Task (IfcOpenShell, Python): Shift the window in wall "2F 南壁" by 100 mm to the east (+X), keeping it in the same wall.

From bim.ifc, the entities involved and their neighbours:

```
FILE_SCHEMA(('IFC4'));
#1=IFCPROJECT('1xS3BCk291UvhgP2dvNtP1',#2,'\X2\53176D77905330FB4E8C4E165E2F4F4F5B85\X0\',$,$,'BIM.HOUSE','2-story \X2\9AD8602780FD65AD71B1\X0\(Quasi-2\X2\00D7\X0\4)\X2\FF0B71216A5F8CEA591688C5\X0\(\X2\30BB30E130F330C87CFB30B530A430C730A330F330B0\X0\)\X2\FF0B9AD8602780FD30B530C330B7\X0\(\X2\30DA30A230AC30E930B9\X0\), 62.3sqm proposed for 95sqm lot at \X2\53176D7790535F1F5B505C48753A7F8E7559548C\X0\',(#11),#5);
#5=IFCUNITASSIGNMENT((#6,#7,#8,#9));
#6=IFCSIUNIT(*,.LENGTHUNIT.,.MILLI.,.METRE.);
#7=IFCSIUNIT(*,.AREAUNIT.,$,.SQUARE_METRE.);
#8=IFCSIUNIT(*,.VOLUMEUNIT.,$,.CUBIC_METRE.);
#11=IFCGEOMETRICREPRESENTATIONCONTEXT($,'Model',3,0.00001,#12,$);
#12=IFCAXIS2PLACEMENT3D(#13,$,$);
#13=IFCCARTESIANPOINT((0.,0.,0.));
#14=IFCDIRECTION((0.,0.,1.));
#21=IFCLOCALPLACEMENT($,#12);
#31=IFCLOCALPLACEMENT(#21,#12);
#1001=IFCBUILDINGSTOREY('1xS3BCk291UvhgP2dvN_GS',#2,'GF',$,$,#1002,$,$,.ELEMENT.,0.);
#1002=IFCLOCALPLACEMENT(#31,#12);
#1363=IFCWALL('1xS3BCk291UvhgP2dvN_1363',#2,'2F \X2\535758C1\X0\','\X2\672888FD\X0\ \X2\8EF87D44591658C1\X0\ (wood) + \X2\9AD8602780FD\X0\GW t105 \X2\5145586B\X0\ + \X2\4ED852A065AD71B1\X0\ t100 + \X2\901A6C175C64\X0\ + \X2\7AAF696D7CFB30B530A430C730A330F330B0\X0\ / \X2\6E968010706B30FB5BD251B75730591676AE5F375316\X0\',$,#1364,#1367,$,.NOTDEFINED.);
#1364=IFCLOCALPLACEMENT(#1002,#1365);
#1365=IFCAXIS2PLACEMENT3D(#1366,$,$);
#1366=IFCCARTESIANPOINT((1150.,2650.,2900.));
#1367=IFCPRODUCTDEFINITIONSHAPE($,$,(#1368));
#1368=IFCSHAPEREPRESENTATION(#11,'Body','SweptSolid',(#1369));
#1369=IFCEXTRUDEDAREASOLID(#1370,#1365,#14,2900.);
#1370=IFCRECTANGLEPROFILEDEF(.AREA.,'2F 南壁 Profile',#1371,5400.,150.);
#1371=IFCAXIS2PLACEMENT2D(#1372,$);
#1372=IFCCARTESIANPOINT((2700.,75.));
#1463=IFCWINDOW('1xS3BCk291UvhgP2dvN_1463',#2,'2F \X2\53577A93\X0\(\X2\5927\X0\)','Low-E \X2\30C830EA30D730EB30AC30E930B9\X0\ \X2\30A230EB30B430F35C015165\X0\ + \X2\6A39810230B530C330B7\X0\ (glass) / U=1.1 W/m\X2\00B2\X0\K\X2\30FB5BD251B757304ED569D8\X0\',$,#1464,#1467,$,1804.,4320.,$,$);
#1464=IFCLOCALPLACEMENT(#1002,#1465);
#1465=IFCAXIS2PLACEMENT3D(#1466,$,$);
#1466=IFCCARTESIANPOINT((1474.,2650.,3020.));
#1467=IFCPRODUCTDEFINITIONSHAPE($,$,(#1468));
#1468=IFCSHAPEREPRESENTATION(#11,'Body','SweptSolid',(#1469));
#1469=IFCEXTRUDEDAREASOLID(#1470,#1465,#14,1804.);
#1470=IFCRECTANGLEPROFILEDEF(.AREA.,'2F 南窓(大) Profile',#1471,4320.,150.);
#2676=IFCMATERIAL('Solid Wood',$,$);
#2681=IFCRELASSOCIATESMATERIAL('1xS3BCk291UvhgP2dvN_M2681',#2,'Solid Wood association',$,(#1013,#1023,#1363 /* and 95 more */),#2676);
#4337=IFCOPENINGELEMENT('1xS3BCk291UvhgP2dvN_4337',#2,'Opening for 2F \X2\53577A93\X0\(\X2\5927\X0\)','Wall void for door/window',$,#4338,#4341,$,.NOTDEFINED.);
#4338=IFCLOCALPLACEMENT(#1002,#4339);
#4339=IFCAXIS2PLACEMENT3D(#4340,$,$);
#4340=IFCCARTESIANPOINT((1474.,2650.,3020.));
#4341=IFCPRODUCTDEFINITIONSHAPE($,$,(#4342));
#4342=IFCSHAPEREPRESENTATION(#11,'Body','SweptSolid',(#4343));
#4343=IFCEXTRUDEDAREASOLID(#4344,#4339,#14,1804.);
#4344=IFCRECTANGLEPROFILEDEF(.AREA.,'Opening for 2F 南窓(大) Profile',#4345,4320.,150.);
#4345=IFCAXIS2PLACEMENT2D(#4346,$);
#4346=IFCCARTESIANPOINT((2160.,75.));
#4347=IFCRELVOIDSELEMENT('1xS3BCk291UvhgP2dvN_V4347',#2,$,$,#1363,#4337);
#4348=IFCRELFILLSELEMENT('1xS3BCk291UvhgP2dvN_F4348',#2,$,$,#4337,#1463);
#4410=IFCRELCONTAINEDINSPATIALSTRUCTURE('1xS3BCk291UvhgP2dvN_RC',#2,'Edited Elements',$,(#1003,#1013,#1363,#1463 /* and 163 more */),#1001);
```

```python
import ifcopenshell
import ifcopenshell.api.geometry
import ifcopenshell.util.placement

model = ifcopenshell.open("bim.ifc")

window = model.by_guid("1xS3BCk291UvhgP2dvN_1463")
opening = window.FillsVoids[0].RelatingOpeningElement
wall = opening.VoidsElements[0].RelatingBuildingElement

wall_matrix = ifcopenshell.util.placement.get_local_placement(wall.ObjectPlacement)
shift = wall_matrix[:3, 0] * 100.0
before = ifcopenshell.util.placement.get_local_placement(window.ObjectPlacement)[:3, 3].copy()

# The window is not placed relative to its opening, so move both.
for product in (opening, window):
    matrix = ifcopenshell.util.placement.get_local_placement(product.ObjectPlacement)
    matrix[:3, 3] += shift
    ifcopenshell.api.geometry.edit_object_placement(model, product=product, matrix=matrix, is_si=False)

after = ifcopenshell.util.placement.get_local_placement(window.ObjectPlacement)[:3, 3]
print("window moved by", (after - before).round(3) + 0.0)

model.write("bim_updated.ifc")
```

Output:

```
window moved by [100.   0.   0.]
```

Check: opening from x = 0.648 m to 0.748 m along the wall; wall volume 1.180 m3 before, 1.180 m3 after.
